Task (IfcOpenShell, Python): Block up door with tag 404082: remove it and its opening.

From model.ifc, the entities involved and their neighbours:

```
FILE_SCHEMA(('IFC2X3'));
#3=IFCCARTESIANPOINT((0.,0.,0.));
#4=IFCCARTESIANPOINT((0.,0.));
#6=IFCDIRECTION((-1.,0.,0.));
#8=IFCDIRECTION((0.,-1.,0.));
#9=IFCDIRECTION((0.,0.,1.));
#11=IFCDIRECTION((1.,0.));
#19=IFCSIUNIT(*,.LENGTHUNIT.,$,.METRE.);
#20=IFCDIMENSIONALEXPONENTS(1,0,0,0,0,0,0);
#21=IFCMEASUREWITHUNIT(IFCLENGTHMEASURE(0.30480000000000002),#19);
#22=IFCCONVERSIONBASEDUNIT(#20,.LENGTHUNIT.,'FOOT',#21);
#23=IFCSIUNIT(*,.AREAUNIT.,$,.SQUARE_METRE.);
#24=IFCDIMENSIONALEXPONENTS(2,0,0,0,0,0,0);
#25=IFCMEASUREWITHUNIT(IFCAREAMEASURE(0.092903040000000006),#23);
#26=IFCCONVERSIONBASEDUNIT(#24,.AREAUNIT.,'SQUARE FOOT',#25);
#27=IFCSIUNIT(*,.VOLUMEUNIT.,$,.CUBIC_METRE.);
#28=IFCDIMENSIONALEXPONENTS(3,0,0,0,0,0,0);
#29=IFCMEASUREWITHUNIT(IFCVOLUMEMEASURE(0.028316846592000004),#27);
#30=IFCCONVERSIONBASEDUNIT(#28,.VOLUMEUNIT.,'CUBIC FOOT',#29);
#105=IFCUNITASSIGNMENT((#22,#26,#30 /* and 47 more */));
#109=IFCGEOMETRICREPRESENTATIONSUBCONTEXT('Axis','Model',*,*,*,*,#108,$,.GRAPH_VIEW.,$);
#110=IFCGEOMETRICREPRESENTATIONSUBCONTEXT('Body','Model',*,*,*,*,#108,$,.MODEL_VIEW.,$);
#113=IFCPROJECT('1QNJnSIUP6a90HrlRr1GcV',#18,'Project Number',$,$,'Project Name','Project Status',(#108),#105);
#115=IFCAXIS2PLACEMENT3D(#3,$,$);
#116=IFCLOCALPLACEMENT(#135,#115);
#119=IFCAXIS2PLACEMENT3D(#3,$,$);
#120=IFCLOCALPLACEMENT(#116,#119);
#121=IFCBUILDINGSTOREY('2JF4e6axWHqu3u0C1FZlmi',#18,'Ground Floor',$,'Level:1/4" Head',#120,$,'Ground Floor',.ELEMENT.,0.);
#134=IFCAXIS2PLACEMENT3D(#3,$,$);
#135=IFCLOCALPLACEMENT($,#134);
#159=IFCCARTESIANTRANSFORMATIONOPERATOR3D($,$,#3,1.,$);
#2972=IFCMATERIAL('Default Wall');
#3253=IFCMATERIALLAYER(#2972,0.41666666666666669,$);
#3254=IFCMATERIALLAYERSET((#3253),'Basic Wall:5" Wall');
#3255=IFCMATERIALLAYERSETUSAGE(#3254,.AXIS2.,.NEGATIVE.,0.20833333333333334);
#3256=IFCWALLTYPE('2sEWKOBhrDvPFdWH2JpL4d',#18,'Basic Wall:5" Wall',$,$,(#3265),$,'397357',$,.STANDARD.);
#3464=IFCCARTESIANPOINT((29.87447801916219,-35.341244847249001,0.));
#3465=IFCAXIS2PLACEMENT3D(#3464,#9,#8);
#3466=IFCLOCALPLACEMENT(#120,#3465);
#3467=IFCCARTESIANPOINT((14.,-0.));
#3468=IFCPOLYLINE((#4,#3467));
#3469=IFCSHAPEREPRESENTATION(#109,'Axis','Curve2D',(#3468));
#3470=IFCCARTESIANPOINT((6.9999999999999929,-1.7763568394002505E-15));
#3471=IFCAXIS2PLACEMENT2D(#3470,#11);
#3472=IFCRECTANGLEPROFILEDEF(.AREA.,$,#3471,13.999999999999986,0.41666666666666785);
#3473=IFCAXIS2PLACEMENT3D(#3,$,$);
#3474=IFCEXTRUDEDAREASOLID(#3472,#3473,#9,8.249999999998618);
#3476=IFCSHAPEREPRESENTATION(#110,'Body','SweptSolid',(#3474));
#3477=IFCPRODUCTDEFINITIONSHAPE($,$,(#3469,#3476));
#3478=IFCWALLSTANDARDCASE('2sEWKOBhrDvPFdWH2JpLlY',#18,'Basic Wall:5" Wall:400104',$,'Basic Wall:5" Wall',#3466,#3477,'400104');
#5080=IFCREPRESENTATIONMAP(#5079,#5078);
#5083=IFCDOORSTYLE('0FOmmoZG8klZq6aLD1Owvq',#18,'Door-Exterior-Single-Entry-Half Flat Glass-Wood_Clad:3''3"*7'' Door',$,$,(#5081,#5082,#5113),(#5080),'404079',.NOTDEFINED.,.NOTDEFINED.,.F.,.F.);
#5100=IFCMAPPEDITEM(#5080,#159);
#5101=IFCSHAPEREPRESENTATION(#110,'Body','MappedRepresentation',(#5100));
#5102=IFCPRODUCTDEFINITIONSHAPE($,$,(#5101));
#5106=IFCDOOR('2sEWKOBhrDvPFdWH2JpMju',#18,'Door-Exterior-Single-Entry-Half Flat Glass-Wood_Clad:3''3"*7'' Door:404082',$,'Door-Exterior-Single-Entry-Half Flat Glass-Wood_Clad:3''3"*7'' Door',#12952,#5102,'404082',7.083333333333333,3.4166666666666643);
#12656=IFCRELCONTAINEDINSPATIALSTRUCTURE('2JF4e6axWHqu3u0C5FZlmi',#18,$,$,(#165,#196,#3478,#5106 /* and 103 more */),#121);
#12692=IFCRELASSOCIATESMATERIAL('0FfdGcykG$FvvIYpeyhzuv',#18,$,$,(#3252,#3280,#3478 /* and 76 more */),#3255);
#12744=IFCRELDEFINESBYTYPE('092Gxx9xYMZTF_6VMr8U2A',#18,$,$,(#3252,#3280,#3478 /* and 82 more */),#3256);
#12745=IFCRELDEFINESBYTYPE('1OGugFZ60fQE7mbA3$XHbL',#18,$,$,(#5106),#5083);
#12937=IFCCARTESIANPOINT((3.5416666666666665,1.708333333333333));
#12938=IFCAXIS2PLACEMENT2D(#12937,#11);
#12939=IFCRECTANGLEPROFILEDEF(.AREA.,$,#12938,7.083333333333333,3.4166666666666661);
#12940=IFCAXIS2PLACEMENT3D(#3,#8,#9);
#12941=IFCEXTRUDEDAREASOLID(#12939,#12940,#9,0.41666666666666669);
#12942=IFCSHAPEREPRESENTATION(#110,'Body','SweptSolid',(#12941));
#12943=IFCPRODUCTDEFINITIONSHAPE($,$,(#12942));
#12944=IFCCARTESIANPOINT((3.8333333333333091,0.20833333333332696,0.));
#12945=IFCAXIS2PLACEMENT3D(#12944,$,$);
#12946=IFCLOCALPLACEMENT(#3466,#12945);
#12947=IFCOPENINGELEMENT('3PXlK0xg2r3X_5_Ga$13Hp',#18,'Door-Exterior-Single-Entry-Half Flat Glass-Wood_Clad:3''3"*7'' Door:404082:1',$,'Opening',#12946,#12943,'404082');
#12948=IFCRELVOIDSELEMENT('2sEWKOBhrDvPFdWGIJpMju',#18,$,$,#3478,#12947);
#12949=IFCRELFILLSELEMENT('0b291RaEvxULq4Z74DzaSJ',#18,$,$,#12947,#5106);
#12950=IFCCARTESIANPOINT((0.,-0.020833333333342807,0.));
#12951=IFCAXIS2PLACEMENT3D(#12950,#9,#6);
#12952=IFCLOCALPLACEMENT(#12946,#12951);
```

```python
import ifcopenshell
import ifcopenshell.api.feature
import ifcopenshell.api.root
import ifcopenshell.geom
import ifcopenshell.util.shape

model = ifcopenshell.open("model.ifc")
settings = ifcopenshell.geom.settings()


def volume(element):
    """Net volume in cubic metres, openings subtracted."""
    shape = ifcopenshell.geom.create_shape(settings, element)
    return ifcopenshell.util.shape.get_volume(shape.geometry)


door = model.by_id(5106)
opening = door.FillsVoids[0].RelatingOpeningElement
wall = opening.VoidsElements[0].RelatingBuildingElement
before = volume(wall)

ifcopenshell.api.root.remove_product(model, product=door)
ifcopenshell.api.feature.remove_feature(model, feature=opening)

after = volume(wall)

print(f"wall volume {before:.3f} -> {after:.3f} m3")

model.write("model_updated.ifc")
```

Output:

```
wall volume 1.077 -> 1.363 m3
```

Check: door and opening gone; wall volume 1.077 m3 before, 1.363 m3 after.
